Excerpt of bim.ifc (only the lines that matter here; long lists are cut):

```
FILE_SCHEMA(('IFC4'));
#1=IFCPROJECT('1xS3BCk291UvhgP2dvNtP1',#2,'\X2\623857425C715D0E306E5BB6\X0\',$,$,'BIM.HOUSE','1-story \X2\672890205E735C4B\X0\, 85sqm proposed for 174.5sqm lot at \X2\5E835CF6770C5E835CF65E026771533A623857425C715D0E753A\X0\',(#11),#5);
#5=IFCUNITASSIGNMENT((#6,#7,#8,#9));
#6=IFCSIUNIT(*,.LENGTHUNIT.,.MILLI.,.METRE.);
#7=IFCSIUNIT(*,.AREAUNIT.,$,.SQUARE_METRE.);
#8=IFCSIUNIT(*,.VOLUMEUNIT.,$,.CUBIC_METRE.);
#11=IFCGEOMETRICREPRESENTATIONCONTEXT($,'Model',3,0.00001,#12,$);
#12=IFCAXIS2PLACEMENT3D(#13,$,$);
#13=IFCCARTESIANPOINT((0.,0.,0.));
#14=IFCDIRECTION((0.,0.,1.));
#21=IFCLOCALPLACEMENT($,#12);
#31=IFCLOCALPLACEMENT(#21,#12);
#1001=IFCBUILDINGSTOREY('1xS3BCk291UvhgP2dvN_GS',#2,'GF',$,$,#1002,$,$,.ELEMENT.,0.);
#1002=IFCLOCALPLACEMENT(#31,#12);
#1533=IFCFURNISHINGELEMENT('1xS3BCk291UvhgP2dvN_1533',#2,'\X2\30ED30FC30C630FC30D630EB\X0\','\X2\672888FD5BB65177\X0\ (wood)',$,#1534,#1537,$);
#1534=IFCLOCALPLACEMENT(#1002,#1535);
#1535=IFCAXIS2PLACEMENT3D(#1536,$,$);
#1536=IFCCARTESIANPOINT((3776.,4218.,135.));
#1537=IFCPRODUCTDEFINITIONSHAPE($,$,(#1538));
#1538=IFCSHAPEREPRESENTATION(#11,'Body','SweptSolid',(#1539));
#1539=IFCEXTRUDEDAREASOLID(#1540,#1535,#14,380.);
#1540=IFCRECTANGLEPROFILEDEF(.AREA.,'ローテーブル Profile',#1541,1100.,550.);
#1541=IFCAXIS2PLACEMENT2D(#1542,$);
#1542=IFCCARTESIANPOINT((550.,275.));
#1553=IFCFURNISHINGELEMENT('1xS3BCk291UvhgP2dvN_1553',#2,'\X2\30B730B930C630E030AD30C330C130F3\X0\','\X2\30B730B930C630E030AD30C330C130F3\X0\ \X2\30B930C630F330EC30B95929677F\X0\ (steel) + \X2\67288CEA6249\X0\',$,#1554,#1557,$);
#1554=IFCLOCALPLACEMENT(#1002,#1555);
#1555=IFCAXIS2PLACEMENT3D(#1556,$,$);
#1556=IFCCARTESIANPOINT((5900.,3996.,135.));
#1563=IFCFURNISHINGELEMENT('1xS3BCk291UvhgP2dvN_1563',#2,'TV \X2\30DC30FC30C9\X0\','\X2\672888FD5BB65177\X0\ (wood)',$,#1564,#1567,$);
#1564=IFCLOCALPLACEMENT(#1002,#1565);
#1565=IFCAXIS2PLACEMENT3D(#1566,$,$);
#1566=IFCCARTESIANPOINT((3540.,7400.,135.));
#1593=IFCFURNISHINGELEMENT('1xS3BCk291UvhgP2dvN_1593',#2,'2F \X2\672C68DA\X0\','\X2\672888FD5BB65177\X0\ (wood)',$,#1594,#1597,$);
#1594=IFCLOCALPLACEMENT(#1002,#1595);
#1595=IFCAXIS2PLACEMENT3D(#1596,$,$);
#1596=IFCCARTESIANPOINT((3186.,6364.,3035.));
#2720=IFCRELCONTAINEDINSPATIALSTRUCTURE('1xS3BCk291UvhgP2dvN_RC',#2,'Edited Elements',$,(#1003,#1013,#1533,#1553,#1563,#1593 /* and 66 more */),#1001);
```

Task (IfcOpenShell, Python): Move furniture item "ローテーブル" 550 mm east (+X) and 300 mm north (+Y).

```python
import ifcopenshell
import ifcopenshell.api.geometry
import ifcopenshell.util.placement

model = ifcopenshell.open("bim.ifc")

item = model.by_id(1533)
matrix = ifcopenshell.util.placement.get_local_placement(item.ObjectPlacement)
matrix[0, 3] += 550.0
matrix[1, 3] += 300.0
ifcopenshell.api.geometry.edit_object_placement(model, product=item, matrix=matrix, is_si=False)

print(ifcopenshell.util.placement.get_local_placement(item.ObjectPlacement).round(3) + 0.0)

model.write("bim_v2.ifc")
```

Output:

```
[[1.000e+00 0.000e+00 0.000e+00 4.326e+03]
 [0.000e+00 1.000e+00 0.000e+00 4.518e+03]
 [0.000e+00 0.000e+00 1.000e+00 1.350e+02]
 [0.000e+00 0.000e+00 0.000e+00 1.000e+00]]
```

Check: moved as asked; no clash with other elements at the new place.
